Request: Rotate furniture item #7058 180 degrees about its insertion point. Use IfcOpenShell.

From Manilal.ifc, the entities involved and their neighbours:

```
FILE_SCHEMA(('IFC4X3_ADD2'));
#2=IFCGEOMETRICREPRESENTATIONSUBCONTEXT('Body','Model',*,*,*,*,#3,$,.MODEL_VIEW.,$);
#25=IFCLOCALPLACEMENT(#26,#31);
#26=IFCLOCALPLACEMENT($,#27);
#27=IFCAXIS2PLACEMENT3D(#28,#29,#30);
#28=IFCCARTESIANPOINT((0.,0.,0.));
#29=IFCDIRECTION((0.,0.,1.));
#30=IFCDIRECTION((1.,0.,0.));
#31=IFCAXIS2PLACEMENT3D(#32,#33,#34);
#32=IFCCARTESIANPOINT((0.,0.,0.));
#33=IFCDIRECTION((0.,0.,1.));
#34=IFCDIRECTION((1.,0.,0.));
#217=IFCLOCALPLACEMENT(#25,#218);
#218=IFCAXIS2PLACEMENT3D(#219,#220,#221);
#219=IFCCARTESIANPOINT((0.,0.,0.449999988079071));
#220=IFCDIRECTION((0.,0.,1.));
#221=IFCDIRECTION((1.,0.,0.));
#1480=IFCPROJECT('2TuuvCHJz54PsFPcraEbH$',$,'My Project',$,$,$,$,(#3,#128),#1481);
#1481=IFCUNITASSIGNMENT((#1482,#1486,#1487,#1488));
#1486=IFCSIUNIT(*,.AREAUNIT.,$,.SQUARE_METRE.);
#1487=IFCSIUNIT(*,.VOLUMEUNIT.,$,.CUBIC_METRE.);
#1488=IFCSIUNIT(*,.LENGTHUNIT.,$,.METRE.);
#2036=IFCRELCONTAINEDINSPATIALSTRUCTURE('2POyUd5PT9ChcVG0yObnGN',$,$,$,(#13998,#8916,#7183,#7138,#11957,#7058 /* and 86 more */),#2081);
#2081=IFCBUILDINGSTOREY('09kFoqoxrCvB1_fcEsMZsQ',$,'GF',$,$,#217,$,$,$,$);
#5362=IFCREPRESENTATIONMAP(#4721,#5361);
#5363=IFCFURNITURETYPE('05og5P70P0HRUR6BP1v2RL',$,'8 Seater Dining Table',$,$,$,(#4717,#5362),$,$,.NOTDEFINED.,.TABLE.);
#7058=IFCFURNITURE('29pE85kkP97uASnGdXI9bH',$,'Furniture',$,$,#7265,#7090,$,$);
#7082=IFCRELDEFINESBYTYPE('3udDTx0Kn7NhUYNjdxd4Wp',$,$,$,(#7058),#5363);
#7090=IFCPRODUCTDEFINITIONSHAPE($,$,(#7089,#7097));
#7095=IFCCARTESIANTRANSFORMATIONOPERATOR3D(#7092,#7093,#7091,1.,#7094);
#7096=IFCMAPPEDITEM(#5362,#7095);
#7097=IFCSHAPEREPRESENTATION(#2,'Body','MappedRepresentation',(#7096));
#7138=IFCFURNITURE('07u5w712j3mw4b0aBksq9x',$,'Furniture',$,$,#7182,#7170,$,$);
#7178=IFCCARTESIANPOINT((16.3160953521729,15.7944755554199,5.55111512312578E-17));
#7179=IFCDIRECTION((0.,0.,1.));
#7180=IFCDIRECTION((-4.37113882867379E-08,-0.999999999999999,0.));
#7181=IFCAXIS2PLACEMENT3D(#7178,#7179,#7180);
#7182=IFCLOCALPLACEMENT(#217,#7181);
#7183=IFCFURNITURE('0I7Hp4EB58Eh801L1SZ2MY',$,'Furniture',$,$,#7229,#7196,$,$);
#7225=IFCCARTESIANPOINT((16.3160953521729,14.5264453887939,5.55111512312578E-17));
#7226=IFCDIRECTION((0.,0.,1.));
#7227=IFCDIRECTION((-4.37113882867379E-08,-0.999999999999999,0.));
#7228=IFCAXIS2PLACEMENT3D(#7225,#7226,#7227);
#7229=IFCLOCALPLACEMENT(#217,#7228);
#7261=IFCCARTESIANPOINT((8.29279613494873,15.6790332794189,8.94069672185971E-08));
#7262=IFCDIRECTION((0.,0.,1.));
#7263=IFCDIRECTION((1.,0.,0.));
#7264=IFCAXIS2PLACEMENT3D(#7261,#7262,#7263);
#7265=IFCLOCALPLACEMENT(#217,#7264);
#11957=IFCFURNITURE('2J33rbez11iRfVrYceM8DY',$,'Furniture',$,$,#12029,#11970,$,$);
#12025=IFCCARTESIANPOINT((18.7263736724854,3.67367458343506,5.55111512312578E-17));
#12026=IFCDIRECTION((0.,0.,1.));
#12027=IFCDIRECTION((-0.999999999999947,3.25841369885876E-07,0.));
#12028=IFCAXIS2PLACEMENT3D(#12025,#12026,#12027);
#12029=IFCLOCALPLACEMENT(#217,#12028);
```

```python
import ifcopenshell
import ifcopenshell.api.geometry
import ifcopenshell.util.placement

model = ifcopenshell.open("Manilal.ifc")

item = model.by_guid("29pE85kkP97uASnGdXI9bH")
matrix = ifcopenshell.util.placement.get_local_placement(item.ObjectPlacement)
matrix = matrix @ ifcopenshell.util.placement.rotation(180, "Z")
ifcopenshell.api.geometry.edit_object_placement(model, product=item, matrix=matrix, is_si=False)

print(ifcopenshell.util.placement.get_local_placement(item.ObjectPlacement).round(3) + 0.0)

model.write("Manilal_v2.ifc")
```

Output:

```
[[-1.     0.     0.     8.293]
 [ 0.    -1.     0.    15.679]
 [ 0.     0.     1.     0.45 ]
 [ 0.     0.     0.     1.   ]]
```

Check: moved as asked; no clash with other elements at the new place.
